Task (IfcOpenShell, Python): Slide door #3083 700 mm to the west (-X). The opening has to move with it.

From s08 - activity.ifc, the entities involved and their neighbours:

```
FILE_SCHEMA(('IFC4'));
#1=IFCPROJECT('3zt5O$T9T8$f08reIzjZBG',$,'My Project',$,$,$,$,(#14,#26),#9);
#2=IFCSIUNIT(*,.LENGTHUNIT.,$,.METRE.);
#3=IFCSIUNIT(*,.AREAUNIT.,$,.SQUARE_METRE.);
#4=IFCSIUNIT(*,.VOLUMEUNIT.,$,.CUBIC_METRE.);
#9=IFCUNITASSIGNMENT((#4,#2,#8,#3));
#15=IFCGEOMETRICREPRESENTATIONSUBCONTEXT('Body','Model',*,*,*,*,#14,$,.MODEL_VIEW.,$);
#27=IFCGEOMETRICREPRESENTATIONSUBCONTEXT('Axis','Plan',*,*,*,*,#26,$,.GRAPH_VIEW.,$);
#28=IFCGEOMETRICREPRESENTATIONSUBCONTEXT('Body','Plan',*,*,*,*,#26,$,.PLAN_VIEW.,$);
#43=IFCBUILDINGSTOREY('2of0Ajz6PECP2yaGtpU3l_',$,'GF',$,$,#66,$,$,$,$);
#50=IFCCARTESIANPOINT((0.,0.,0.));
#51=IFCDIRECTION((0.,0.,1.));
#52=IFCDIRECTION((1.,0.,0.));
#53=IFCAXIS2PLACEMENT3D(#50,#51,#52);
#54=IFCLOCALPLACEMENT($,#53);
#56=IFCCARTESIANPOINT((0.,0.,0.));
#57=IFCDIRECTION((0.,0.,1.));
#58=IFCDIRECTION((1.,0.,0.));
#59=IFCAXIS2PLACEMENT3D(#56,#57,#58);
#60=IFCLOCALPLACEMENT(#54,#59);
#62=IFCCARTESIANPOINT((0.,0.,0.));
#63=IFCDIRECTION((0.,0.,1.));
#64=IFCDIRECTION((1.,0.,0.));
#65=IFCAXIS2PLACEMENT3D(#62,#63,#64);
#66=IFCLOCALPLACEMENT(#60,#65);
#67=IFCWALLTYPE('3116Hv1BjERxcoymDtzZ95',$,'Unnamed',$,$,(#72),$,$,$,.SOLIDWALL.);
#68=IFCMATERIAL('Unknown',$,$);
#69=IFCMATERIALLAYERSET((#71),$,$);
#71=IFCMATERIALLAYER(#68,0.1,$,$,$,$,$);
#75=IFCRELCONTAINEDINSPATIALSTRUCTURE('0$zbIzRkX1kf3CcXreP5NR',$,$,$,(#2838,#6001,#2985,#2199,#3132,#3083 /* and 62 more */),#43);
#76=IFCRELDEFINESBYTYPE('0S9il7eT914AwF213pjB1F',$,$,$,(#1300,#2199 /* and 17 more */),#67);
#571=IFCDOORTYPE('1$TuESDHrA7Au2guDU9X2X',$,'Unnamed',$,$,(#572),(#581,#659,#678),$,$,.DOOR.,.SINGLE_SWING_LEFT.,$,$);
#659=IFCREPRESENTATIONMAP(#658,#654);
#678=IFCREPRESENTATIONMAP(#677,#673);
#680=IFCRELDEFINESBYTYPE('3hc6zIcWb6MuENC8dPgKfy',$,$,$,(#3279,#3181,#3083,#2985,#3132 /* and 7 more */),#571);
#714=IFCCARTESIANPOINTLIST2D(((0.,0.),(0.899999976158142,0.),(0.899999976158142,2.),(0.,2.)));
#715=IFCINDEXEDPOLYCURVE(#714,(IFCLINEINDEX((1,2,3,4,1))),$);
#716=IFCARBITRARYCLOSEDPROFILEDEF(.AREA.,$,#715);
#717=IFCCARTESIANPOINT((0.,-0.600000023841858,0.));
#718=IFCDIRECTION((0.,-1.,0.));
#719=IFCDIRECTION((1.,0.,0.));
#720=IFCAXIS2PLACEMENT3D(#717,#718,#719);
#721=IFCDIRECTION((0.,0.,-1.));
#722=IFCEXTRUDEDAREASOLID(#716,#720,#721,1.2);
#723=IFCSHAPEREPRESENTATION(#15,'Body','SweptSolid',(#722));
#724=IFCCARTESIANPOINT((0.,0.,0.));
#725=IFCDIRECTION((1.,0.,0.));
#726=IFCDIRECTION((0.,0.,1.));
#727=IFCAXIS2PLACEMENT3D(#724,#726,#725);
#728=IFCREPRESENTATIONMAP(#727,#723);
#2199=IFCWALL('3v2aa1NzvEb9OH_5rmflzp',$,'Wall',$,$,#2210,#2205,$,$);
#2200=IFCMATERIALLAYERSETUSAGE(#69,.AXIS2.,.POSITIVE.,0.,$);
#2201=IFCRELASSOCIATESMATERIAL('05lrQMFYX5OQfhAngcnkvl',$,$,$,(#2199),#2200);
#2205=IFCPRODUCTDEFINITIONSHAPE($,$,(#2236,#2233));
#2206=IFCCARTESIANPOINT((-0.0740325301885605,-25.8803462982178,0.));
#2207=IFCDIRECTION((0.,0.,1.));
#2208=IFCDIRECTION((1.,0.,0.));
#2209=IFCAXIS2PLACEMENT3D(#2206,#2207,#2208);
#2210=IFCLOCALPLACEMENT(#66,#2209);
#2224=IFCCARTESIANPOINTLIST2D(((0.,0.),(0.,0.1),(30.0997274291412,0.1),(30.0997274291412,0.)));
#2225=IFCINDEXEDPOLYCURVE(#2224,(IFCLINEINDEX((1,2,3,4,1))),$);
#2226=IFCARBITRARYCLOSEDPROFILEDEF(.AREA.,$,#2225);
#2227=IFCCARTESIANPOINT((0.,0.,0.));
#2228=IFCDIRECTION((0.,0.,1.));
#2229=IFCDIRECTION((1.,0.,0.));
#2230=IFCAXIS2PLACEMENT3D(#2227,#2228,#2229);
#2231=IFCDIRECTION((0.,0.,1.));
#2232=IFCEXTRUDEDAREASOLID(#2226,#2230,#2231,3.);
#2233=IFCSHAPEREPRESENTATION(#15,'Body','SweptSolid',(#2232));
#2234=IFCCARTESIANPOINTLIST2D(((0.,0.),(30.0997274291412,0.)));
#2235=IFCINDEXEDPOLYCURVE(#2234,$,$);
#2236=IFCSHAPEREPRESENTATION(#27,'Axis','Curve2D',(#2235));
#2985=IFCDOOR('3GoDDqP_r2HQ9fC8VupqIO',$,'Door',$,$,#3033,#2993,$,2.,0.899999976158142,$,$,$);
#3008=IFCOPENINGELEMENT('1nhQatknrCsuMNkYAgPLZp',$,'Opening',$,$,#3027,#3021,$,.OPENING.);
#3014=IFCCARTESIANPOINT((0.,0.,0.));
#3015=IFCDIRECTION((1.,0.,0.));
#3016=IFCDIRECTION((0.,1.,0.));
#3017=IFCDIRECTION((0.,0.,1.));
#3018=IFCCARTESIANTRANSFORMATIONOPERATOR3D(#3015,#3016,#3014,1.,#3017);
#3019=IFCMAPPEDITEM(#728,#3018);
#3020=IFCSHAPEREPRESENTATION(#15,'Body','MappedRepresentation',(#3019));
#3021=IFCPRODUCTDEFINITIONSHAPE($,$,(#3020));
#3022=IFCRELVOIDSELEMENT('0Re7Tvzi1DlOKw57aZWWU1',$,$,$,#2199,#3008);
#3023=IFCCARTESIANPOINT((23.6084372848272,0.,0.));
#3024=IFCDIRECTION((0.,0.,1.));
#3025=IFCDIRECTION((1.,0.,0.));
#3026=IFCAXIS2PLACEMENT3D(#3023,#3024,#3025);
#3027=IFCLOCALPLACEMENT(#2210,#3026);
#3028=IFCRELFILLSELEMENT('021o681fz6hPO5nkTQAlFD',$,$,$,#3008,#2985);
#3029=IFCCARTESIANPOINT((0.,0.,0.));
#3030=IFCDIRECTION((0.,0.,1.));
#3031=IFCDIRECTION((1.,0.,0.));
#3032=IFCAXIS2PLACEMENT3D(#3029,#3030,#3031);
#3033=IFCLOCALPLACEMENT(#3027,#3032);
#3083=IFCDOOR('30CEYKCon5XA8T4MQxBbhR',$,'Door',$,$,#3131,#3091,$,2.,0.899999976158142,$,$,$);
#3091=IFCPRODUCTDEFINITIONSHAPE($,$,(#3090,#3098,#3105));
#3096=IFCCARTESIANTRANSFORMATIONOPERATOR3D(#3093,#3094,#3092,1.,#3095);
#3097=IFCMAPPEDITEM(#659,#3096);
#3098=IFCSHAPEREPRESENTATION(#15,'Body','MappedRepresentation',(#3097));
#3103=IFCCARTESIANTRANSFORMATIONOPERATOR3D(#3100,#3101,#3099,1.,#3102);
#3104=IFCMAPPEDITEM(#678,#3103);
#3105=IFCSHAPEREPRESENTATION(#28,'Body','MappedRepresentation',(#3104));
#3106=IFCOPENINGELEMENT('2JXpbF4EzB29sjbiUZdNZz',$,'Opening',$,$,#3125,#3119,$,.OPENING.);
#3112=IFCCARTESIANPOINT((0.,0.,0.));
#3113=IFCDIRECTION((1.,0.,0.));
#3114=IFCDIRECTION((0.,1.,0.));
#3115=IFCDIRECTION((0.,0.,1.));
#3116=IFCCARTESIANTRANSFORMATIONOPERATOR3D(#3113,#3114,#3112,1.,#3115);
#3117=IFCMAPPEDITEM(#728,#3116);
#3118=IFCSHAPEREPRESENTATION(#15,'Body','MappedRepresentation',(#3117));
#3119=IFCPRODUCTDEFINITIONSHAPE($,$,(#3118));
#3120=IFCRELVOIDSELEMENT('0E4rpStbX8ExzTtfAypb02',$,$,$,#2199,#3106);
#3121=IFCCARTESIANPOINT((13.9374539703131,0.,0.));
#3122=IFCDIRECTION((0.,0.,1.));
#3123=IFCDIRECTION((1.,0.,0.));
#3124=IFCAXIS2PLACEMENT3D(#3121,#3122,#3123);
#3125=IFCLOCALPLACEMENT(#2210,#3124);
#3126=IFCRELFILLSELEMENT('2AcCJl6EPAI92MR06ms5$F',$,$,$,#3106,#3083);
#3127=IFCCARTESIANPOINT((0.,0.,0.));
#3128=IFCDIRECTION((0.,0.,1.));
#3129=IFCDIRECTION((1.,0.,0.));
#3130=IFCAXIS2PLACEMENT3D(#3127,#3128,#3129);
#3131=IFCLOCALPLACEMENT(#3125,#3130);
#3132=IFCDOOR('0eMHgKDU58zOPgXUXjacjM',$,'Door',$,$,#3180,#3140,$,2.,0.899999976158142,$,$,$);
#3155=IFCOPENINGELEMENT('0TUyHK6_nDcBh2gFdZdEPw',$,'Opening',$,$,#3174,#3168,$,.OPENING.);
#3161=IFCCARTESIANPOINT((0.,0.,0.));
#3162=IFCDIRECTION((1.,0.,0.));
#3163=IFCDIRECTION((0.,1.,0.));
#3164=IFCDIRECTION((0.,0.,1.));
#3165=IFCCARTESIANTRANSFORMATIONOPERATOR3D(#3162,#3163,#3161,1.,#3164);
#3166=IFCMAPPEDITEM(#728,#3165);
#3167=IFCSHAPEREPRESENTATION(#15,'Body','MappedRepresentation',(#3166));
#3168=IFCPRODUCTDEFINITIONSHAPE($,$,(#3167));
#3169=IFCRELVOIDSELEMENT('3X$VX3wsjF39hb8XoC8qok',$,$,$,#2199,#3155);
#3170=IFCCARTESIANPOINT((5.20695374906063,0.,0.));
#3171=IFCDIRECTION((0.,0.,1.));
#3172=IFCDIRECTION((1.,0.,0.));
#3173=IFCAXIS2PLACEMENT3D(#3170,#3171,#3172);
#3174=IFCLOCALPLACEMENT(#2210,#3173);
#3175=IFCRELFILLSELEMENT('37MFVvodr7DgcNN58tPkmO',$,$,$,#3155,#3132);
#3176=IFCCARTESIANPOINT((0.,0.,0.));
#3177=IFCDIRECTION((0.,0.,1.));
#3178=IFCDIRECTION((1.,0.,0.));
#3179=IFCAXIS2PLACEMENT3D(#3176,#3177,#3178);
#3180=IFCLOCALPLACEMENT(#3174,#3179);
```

```python
import ifcopenshell
import ifcopenshell.api.geometry
import ifcopenshell.util.placement
import ifcopenshell.util.unit

model = ifcopenshell.open("s08 - activity.ifc")
unit_scale = ifcopenshell.util.unit.calculate_unit_scale(model)

door = model.by_guid("30CEYKCon5XA8T4MQxBbhR")
opening = door.FillsVoids[0].RelatingOpeningElement
wall = opening.VoidsElements[0].RelatingBuildingElement

wall_matrix = ifcopenshell.util.placement.get_local_placement(wall.ObjectPlacement)
shift = wall_matrix[:3, 0] * -0.7 / unit_scale
before = ifcopenshell.util.placement.get_local_placement(door.ObjectPlacement)[:3, 3].copy()

# The door is placed relative to its opening, so it follows when the opening moves.
matrix = ifcopenshell.util.placement.get_local_placement(opening.ObjectPlacement)
matrix[:3, 3] += shift
ifcopenshell.api.geometry.edit_object_placement(
    model, product=opening, matrix=matrix, is_si=False, should_transform_children=True
)

after = ifcopenshell.util.placement.get_local_placement(door.ObjectPlacement)[:3, 3]
print("door moved by", (after - before).round(3) + 0.0)

model.write("s08 - activity_v2.ifc")
```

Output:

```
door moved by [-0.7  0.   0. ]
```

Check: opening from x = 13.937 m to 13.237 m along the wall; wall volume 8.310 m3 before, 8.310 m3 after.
